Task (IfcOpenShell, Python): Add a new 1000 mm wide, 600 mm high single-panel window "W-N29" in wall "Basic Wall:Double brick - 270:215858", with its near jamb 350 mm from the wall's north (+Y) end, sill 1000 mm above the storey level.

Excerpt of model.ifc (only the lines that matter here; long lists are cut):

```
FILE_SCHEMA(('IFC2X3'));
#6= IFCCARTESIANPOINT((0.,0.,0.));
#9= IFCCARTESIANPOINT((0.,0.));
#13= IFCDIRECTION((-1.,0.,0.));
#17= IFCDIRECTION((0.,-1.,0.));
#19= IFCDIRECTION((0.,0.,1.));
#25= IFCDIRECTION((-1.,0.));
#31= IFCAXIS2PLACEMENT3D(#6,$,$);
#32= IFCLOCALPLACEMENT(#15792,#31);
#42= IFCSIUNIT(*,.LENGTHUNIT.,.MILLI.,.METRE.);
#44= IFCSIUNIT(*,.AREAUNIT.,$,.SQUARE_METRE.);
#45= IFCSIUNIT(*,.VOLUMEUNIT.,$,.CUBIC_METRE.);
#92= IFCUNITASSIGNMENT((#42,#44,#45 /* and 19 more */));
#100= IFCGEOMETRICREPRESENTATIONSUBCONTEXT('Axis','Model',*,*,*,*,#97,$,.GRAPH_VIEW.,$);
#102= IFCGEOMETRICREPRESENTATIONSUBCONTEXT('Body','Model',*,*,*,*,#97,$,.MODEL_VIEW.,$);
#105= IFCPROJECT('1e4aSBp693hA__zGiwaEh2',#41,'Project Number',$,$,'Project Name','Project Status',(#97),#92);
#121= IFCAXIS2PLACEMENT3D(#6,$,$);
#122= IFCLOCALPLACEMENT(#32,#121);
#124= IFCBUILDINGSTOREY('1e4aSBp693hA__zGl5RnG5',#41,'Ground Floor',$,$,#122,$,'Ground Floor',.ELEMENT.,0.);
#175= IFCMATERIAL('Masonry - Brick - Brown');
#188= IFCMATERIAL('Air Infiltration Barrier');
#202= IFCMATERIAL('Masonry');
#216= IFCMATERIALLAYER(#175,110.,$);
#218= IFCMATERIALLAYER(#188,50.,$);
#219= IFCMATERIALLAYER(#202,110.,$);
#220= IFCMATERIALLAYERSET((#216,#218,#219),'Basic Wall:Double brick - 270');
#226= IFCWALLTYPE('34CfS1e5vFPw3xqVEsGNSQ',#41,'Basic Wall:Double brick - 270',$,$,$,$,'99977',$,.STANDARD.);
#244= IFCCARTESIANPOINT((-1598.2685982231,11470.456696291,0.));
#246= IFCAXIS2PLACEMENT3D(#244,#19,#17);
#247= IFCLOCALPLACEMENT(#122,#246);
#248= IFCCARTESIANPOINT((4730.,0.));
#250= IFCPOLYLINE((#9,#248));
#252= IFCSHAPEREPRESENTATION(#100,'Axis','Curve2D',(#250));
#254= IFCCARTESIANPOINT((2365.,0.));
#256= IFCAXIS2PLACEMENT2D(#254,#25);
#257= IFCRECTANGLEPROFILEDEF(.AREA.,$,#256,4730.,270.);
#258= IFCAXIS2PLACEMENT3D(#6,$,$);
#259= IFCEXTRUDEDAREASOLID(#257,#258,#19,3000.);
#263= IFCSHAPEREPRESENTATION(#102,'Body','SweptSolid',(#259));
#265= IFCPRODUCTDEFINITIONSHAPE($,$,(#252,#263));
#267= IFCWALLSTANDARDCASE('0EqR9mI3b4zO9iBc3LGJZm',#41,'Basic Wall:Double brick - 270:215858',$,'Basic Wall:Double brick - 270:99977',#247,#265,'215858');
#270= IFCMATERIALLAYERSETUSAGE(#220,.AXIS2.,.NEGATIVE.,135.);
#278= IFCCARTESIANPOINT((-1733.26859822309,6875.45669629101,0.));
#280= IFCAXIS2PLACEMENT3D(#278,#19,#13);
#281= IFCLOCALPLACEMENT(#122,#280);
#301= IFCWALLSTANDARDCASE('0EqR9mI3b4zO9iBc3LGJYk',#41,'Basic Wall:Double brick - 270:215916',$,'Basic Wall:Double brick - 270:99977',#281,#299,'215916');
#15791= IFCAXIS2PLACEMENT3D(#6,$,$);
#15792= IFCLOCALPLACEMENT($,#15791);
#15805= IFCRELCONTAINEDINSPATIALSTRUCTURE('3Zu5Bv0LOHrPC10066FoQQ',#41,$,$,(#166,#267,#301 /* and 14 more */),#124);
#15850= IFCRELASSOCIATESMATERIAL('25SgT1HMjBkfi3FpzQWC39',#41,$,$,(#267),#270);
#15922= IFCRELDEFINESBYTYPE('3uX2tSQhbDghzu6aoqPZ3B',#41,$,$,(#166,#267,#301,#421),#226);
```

```python
import numpy as np
import ifcopenshell
import ifcopenshell.api.feature
import ifcopenshell.api.geometry
import ifcopenshell.api.root
import ifcopenshell.api.spatial
import ifcopenshell.api.type
import ifcopenshell.geom
import ifcopenshell.util.element
import ifcopenshell.util.placement
import ifcopenshell.util.representation
import ifcopenshell.util.shape
import ifcopenshell.util.unit

model = ifcopenshell.open("model.ifc")
unit_scale = ifcopenshell.util.unit.calculate_unit_scale(model)
settings = ifcopenshell.geom.settings()


def volume(element):
    """Net volume in cubic metres, openings subtracted."""
    shape = ifcopenshell.geom.create_shape(settings, element)
    return ifcopenshell.util.shape.get_volume(shape.geometry)


wall = model.by_guid("0EqR9mI3b4zO9iBc3LGJZm")
storey = ifcopenshell.util.element.get_container(wall, ifc_class="IfcBuildingStorey")
context = ifcopenshell.util.representation.get_context(model, "Model", "Body", "MODEL_VIEW")
before = volume(wall)

width, height, from_end, sill = 1, 0.6, 0.35, 1  # metres

# The wall runs along its own X axis, and the end named is its -X end.
wall_shape = ifcopenshell.geom.create_shape(settings, wall)
x, y, z = ifcopenshell.util.shape.get_vertices(wall_shape.geometry).T
start = x.min() + from_end
face, thickness = float(y.min()), float(y.max() - y.min())
wall_matrix = ifcopenshell.util.placement.get_local_placement(wall.ObjectPlacement)
level = ifcopenshell.util.placement.get_local_placement(storey.ObjectPlacement)[2, 3]


def in_wall(x, y):
    """Placement at x, y metres in the wall's axes, at sill height."""
    matrix = wall_matrix.copy()
    matrix[:, 3] = wall_matrix @ np.array([x / unit_scale, y / unit_scale, 0.0, 1.0])
    matrix[2, 3] = level + sill / unit_scale
    return matrix


# Opening: a box that overshoots both wall faces by 50 mm.
opening = ifcopenshell.api.root.create_entity(model, ifc_class="IfcOpeningElement")
box = ifcopenshell.api.geometry.add_wall_representation(
    model, context=context, length=width, height=height, thickness=thickness + 0.1
)
ifcopenshell.api.geometry.assign_representation(model, product=opening, representation=box)
ifcopenshell.api.geometry.edit_object_placement(model, product=opening, matrix=in_wall(start, face - 0.05), is_si=False)
ifcopenshell.api.feature.add_feature(model, feature=opening, element=wall)

window = ifcopenshell.api.root.create_entity(model, ifc_class="IfcWindow", name="W-N29")
window.OverallWidth, window.OverallHeight = width / unit_scale, height / unit_scale
body = ifcopenshell.api.geometry.add_window_representation(
    model,
    context=context,
    overall_width=window.OverallWidth,
    overall_height=window.OverallHeight,
    partition_type="SINGLE_PANEL",
)
ifcopenshell.api.geometry.assign_representation(model, product=window, representation=body)
ifcopenshell.api.spatial.assign_container(model, products=[window], relating_structure=storey)
fills = ifcopenshell.api.feature.add_filling(model, opening=opening, element=window)
fills.OwnerHistory = window.OwnerHistory  # required in IFC2X3

# IFC2X3 keeps the operation on the window style.
style = ifcopenshell.api.root.create_entity(model, ifc_class="IfcWindowStyle", name="W-N29")
style.OperationType, style.ConstructionType = "SINGLE_PANEL", "NOTDEFINED"
style.ParameterTakesPrecedence = style.Sizeable = False
ifcopenshell.api.type.assign_type(model, related_objects=[window], relating_type=style)

# Centre the window in the wall's thickness.
ifcopenshell.api.geometry.edit_object_placement(model, product=window, matrix=in_wall(start, face), is_si=False)
window_shape = ifcopenshell.geom.create_shape(settings, window)
depth = ifcopenshell.util.shape.get_vertices(window_shape.geometry)[:, 1]
offset = face + thickness / 2 - (depth.min() + depth.max()) / 2
ifcopenshell.api.geometry.edit_object_placement(model, product=window, matrix=in_wall(start, offset), is_si=False)

after = volume(wall)

print(f"wall volume {before:.3f} -> {after:.3f} m3")

model.write("model_edited.ifc")
```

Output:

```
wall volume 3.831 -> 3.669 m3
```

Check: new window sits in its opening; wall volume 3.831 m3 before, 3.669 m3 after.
